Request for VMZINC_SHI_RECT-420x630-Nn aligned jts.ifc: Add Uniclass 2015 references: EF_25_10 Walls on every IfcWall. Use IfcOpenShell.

First a look at what the model holds.

```python
import ifcopenshell

model = ifcopenshell.open("VMZINC_SHI_RECT-420x630-Nn aligned jts.ifc")
print(model.schema)
print("classifications:", [c.Name for c in model.by_type("IfcClassification")])
for ifc_class in ("IfcDoor", "IfcRoof", "IfcStair", "IfcWall", "IfcWindow"):
    print(ifc_class, len(model.by_type(ifc_class)))
```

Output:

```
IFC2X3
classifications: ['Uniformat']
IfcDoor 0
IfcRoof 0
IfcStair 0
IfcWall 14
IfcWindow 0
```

```python
import ifcopenshell
import ifcopenshell.api.classification

model = ifcopenshell.open("VMZINC_SHI_RECT-420x630-Nn aligned jts.ifc")

# IFC2X3 requires Source and Edition and has no link from the project to the system.
system = model.create_entity("IfcClassification", Source="NBS", Edition="2015", Name="Uniclass 2015")

codes = {
    "IfcWall": ("EF_25_10", "Walls"),
}
for ifc_class, (code, name) in codes.items():
    products = model.by_type(ifc_class)
    ifcopenshell.api.classification.add_reference(
        model, products=products, classification=system, identification=code, name=name
    )
    print(code, len(products))

model.write("VMZINC_SHI_RECT-420x630-Nn aligned jts_updated.ifc")
```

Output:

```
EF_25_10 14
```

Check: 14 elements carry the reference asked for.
